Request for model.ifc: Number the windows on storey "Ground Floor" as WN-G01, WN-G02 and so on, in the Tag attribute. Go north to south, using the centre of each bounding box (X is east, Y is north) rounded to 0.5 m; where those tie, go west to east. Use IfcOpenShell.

First a look at what the model holds.

```python
import ifcopenshell
import ifcopenshell.util.element
import ifcopenshell.util.placement

model = ifcopenshell.open("model.ifc")
print(model.schema)
storey = next(s for s in model.by_type("IfcBuildingStorey") if s.Name == "Ground Floor")
windows = [e for e in ifcopenshell.util.element.get_decomposition(storey) if e.is_a("IfcWindow")]
for e in sorted(windows, key=lambda e: e.id()):
    origin = ifcopenshell.util.placement.get_local_placement(e.ObjectPlacement)[:3, 3]
    print(e.id(), e.Tag, e.Name, origin.round(2) + 0.0, sep=" | ")
```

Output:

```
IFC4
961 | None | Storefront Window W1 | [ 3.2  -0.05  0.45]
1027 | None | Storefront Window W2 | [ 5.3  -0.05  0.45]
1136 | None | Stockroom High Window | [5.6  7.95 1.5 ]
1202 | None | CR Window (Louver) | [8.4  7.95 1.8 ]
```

```python
import ifcopenshell
import ifcopenshell.geom
import ifcopenshell.util.element
import ifcopenshell.util.shape

model = ifcopenshell.open("model.ifc")
settings = ifcopenshell.geom.settings()
settings.set("use-world-coords", True)


def centre(element):
    shape = ifcopenshell.geom.create_shape(settings, element)
    return ifcopenshell.util.shape.get_bbox_centroid(shape.geometry)


storey = next(s for s in model.by_type("IfcBuildingStorey") if s.Name == "Ground Floor")
windows = [e for e in ifcopenshell.util.element.get_decomposition(storey) if e.is_a("IfcWindow")]

# Insertion points can sit at a corner or the storey origin, so sort by the geometry (in metres).
centres = {e: centre(e) for e in windows}
windows.sort(key=lambda e: (-round(centres[e][1] / 0.5), centres[e][0]))

for i, e in enumerate(windows, start=1):
    number = f"WN-G{i:02d}"
    e.Tag = number
    print(e.id(), number)

model.write("model_updated.ifc")
```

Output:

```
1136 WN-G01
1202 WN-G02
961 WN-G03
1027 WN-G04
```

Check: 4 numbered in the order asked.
